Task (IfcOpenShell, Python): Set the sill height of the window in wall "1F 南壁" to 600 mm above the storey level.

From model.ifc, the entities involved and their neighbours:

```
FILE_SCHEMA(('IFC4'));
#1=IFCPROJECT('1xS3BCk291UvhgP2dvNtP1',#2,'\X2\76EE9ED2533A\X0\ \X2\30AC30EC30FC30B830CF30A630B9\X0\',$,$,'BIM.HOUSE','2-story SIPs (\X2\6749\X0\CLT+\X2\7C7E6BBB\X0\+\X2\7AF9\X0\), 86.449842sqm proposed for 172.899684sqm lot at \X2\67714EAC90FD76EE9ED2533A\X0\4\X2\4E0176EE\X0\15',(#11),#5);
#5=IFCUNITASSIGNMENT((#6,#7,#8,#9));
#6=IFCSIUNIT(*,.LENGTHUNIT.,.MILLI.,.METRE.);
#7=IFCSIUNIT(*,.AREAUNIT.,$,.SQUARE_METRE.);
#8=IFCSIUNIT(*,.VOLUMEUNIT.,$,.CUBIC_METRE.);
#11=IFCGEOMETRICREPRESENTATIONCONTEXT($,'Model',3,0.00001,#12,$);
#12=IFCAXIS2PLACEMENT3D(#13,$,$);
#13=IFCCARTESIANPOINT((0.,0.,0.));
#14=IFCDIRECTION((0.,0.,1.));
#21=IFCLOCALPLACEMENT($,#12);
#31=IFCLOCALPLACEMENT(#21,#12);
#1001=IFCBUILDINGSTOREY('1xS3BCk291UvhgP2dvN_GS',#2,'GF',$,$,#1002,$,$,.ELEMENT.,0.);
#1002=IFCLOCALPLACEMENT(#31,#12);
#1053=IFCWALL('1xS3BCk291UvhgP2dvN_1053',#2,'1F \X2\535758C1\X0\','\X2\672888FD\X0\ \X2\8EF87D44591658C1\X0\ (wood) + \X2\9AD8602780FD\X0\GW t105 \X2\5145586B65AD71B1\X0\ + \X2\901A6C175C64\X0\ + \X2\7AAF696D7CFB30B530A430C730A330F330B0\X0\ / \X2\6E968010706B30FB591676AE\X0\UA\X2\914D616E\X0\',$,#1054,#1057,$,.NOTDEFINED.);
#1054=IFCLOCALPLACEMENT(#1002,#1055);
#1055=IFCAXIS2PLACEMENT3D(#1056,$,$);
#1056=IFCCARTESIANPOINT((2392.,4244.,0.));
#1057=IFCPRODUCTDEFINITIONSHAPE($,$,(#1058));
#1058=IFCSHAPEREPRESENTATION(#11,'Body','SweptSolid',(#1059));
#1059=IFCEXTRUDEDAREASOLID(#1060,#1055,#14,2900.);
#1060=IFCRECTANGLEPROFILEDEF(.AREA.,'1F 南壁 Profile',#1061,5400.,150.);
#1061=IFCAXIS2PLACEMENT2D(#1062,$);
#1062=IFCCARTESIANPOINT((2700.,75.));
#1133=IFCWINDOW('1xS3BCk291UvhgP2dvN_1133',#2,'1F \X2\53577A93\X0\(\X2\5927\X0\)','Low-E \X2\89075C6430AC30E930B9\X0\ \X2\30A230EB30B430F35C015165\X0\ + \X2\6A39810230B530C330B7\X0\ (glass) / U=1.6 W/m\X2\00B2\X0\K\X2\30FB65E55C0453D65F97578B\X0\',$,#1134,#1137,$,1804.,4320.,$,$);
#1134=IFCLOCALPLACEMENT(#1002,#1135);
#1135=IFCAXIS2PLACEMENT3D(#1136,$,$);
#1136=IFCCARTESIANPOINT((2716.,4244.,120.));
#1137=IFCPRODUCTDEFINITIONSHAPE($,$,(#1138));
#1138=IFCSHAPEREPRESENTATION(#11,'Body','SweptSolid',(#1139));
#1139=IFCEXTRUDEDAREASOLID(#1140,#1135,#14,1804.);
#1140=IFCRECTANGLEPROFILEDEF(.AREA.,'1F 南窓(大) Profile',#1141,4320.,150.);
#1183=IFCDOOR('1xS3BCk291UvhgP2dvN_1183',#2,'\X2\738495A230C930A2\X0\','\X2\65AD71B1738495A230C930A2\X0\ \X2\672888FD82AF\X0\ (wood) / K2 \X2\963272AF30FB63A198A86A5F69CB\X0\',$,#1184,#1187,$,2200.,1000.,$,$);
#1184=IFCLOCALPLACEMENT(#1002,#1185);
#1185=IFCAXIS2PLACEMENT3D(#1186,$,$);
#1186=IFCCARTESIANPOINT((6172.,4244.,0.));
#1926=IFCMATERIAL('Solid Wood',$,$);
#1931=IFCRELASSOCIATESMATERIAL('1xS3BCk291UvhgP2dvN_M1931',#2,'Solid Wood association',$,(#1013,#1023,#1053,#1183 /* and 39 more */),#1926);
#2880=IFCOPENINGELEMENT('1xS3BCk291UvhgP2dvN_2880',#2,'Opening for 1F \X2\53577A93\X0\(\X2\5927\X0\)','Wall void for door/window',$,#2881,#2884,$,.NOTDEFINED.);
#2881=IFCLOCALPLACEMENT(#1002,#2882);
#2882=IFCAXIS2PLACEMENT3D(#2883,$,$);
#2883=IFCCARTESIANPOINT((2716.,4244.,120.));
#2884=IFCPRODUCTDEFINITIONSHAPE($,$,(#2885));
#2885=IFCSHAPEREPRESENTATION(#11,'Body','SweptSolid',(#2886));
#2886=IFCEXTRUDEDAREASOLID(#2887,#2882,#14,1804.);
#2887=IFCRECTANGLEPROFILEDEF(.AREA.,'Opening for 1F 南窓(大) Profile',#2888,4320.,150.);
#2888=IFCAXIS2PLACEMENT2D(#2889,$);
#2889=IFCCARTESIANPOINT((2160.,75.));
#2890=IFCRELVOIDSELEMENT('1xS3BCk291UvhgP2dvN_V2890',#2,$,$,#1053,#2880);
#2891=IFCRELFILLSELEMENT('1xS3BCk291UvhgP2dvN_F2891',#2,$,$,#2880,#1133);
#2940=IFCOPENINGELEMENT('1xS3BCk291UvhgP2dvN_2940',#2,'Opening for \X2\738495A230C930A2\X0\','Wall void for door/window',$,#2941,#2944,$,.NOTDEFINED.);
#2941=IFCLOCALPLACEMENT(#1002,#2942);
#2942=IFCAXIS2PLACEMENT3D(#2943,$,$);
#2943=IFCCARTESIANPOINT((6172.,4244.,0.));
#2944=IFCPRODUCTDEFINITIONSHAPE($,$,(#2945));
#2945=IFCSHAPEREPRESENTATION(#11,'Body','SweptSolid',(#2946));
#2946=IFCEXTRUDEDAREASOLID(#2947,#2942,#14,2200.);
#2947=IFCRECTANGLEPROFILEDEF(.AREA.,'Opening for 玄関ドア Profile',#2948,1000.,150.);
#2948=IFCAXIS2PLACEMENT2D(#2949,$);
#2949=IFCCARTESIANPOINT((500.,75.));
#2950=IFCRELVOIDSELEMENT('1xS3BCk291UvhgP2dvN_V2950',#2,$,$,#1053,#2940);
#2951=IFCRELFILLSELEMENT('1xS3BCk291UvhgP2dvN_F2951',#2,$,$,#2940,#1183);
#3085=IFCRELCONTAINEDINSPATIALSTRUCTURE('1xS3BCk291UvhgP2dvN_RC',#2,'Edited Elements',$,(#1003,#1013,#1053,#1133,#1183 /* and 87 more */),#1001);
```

```python
import numpy as np
import ifcopenshell
import ifcopenshell.api.geometry
import ifcopenshell.geom
import ifcopenshell.util.element
import ifcopenshell.util.placement
import ifcopenshell.util.shape
import ifcopenshell.util.unit

model = ifcopenshell.open("model.ifc")
unit_scale = ifcopenshell.util.unit.calculate_unit_scale(model)

window = model.by_guid("1xS3BCk291UvhgP2dvN_1133")
opening = window.FillsVoids[0].RelatingOpeningElement
storey = ifcopenshell.util.element.get_container(window, ifc_class="IfcBuildingStorey")
level = ifcopenshell.util.placement.get_local_placement(storey.ObjectPlacement)[2, 3]

# The opening's origin need not be at the sill, so measure its lowest point.
shape = ifcopenshell.geom.create_shape(ifcopenshell.geom.settings(), opening)
bottom = ifcopenshell.util.shape.get_shape_bottom_elevation(shape, shape.geometry) / unit_scale
dz = level + 600.0 - bottom

shift = np.array([0.0, 0.0, dz])
# The window is not placed relative to its opening, so move both.
for product in (opening, window):
    matrix = ifcopenshell.util.placement.get_local_placement(product.ObjectPlacement)
    matrix[:3, 3] += shift
    ifcopenshell.api.geometry.edit_object_placement(model, product=product, matrix=matrix, is_si=False)

print(f"moved by {dz * unit_scale:+.3f} m")

model.write("model_updated.ifc")
```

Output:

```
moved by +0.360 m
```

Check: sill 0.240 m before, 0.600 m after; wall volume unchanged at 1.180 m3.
